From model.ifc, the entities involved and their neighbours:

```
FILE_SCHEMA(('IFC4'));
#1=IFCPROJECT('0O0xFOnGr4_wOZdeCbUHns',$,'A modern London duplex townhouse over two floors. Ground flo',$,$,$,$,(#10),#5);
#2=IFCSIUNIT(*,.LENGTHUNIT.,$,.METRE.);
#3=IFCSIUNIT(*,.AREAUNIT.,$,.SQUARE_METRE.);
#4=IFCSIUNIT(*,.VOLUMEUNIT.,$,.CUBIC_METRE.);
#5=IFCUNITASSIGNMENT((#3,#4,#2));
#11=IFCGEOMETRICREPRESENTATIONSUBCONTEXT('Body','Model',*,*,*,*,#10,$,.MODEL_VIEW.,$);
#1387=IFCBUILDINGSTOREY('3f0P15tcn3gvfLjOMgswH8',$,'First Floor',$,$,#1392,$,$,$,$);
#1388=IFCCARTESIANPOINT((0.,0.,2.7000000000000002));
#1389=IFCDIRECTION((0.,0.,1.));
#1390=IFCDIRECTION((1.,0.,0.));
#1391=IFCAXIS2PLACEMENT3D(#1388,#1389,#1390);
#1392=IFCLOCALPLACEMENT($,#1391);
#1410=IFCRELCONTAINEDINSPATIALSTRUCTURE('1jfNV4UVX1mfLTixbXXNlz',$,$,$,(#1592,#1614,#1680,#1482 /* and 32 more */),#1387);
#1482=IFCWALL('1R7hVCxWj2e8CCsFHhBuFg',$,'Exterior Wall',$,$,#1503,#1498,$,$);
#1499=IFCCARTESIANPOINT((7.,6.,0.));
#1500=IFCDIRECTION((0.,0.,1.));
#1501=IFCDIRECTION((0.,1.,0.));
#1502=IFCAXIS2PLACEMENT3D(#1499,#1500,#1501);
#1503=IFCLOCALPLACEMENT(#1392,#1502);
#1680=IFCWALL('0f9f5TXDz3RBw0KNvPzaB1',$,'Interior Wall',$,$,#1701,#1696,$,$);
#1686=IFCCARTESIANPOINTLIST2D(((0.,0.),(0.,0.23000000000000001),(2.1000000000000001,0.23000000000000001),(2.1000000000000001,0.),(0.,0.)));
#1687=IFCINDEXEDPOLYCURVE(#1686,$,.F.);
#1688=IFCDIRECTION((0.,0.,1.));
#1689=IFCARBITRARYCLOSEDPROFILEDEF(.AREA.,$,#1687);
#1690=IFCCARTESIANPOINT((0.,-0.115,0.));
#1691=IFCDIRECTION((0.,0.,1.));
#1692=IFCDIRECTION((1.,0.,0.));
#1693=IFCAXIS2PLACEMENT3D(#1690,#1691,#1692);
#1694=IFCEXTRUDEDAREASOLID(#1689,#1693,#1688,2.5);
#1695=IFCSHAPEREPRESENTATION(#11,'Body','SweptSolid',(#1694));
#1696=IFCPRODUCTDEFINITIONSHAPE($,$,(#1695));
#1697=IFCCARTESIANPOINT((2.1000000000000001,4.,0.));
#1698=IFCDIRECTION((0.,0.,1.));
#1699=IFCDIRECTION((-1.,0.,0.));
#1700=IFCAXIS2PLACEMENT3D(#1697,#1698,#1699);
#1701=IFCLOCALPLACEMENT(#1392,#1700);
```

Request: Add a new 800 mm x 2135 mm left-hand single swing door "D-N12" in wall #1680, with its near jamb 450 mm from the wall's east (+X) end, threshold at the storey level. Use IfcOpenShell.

```python
import numpy as np
import ifcopenshell
import ifcopenshell.api.feature
import ifcopenshell.api.geometry
import ifcopenshell.api.root
import ifcopenshell.api.spatial
import ifcopenshell.geom
import ifcopenshell.util.element
import ifcopenshell.util.placement
import ifcopenshell.util.representation
import ifcopenshell.util.shape
import ifcopenshell.util.unit

model = ifcopenshell.open("model.ifc")
unit_scale = ifcopenshell.util.unit.calculate_unit_scale(model)
settings = ifcopenshell.geom.settings()


def volume(element):
    """Net volume in cubic metres, openings subtracted."""
    shape = ifcopenshell.geom.create_shape(settings, element)
    return ifcopenshell.util.shape.get_volume(shape.geometry)


wall = model.by_guid("0f9f5TXDz3RBw0KNvPzaB1")
storey = ifcopenshell.util.element.get_container(wall, ifc_class="IfcBuildingStorey")
context = ifcopenshell.util.representation.get_context(model, "Model", "Body", "MODEL_VIEW")
before = volume(wall)

width, height, from_end, sill = 0.8, 2.135, 0.45, 0.0  # metres

# The wall runs along its own X axis, and the end named is its -X end.
wall_shape = ifcopenshell.geom.create_shape(settings, wall)
x, y, z = ifcopenshell.util.shape.get_vertices(wall_shape.geometry).T
start = x.min() + from_end
face, thickness = float(y.min()), float(y.max() - y.min())
wall_matrix = ifcopenshell.util.placement.get_local_placement(wall.ObjectPlacement)
level = ifcopenshell.util.placement.get_local_placement(storey.ObjectPlacement)[2, 3]


def in_wall(x, y):
    """Placement at x, y metres in the wall's axes, at sill height."""
    matrix = wall_matrix.copy()
    matrix[:, 3] = wall_matrix @ np.array([x / unit_scale, y / unit_scale, 0.0, 1.0])
    matrix[2, 3] = level + sill / unit_scale
    return matrix


# Opening: a box that overshoots both wall faces by 50 mm.
opening = ifcopenshell.api.root.create_entity(model, ifc_class="IfcOpeningElement", predefined_type="OPENING")
box = ifcopenshell.api.geometry.add_wall_representation(
    model, context=context, length=width, height=height, thickness=thickness + 0.1
)
ifcopenshell.api.geometry.assign_representation(model, product=opening, representation=box)
ifcopenshell.api.geometry.edit_object_placement(model, product=opening, matrix=in_wall(start, face - 0.05), is_si=False)
ifcopenshell.api.feature.add_feature(model, feature=opening, element=wall)

door = ifcopenshell.api.root.create_entity(model, ifc_class="IfcDoor", name="D-N12", predefined_type="DOOR")
door.OverallWidth, door.OverallHeight = width / unit_scale, height / unit_scale
door.OperationType = "SINGLE_SWING_LEFT"
body = ifcopenshell.api.geometry.add_door_representation(
    model,
    context=context,
    overall_width=door.OverallWidth,
    overall_height=door.OverallHeight,
    operation_type="SINGLE_SWING_LEFT",
    lining_properties={"LiningDepth": thickness / unit_scale, "ThresholdDepth": thickness / unit_scale},
)
ifcopenshell.api.geometry.assign_representation(model, product=door, representation=body)
ifcopenshell.api.spatial.assign_container(model, products=[door], relating_structure=storey)
ifcopenshell.api.feature.add_filling(model, opening=opening, element=door)

# The lining spans the wall, so the door starts at the wall face.
ifcopenshell.api.geometry.edit_object_placement(model, product=door, matrix=in_wall(start, face), is_si=False)

after = volume(wall)

print(f"wall volume {before:.3f} -> {after:.3f} m3")

model.write("model_rev.ifc")
```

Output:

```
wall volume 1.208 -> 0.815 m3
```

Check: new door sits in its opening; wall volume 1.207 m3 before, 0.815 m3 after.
